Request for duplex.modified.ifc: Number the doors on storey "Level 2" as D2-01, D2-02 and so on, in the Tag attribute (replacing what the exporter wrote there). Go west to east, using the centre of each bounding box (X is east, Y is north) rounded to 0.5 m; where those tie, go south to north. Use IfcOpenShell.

First a look at what the model holds.

```python
import ifcopenshell
import ifcopenshell.util.element
import ifcopenshell.util.placement

model = ifcopenshell.open("duplex.modified.ifc")
print(model.schema)
storey = next(s for s in model.by_type("IfcBuildingStorey") if s.Name == "Level 2")
doors = [e for e in ifcopenshell.util.element.get_decomposition(storey) if e.is_a("IfcDoor")]
for e in sorted(doors, key=lambda e: e.id()):
    origin = ifcopenshell.util.placement.get_local_placement(e.ObjectPlacement)[:3, 3]
    print(e.id(), e.Tag, e.Name, origin.round(2) + 0.0, sep=" | ")
```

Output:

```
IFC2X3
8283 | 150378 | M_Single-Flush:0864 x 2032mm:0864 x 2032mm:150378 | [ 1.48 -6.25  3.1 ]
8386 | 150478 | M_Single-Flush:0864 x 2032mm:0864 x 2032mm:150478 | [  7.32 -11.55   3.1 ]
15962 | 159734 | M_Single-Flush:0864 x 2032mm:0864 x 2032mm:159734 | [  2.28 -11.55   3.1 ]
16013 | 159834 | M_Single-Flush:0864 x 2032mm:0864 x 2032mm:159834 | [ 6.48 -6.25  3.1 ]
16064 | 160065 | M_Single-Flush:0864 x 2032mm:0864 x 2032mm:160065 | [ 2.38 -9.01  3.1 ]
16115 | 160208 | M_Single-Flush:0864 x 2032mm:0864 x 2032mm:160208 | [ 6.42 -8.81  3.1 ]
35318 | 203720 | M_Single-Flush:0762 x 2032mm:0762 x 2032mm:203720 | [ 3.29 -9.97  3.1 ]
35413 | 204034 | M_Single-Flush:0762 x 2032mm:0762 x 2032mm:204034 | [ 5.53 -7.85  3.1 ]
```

```python
import ifcopenshell
import ifcopenshell.geom
import ifcopenshell.util.element
import ifcopenshell.util.shape

model = ifcopenshell.open("duplex.modified.ifc")
settings = ifcopenshell.geom.settings()
settings.set("use-world-coords", True)


def centre(element):
    shape = ifcopenshell.geom.create_shape(settings, element)
    return ifcopenshell.util.shape.get_bbox_centroid(shape.geometry)


storey = next(s for s in model.by_type("IfcBuildingStorey") if s.Name == "Level 2")
doors = [e for e in ifcopenshell.util.element.get_decomposition(storey) if e.is_a("IfcDoor")]

# Insertion points can sit at a corner or the storey origin, so sort by the geometry (in metres).
centres = {e: centre(e) for e in doors}
doors.sort(key=lambda e: (round(centres[e][0] / 0.5), centres[e][1]))

for i, e in enumerate(doors, start=1):
    number = f"D2-{i:02d}"
    e.Tag = number
    print(e.id(), number)

model.write("duplex.modified_edited.ifc")
```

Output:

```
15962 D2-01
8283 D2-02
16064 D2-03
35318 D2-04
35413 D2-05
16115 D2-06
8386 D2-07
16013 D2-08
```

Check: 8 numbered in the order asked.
